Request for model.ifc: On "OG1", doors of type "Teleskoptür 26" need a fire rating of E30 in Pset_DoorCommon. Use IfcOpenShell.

First a look at what the model holds.

```python
import ifcopenshell
import ifcopenshell.util.element

model = ifcopenshell.open("model.ifc")
print(model.schema)
storey = next(s for s in model.by_type("IfcBuildingStorey") if s.Name == "OG1")
doors = [e for e in ifcopenshell.util.element.get_decomposition(storey) if e.is_a("IfcDoor")]
seen = {}
for e in doors:
    element_type = ifcopenshell.util.element.get_type(e)
    key = (element_type.Name if element_type != e and element_type else None, ifcopenshell.util.element.get_pset(e, "Pset_DoorCommon", "FireRating"))
    seen[key] = seen.get(key, 0) + 1
for (name, value), count in sorted(seen.items(), key=str):
    print(count, "x", name, "|", value)
```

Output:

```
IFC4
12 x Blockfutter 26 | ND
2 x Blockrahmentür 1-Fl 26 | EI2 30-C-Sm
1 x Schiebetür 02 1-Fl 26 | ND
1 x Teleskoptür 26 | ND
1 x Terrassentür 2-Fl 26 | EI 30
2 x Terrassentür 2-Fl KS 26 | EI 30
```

```python
import ifcopenshell
import ifcopenshell.api.pset
import ifcopenshell.util.element

model = ifcopenshell.open("model.ifc")

storey = next(s for s in model.by_type("IfcBuildingStorey") if s.Name == "OG1")
doors = [e for e in ifcopenshell.util.element.get_decomposition(storey) if e.is_a("IfcDoor")]

count = 0
for e in doors:
    element_type = ifcopenshell.util.element.get_type(e)
    if element_type in (None, e) or element_type.Name != "Teleskoptür 26":
        continue
    # add_pset returns the element's existing set when there is one.
    pset = ifcopenshell.api.pset.add_pset(model, product=e, name="Pset_DoorCommon")
    ifcopenshell.api.pset.edit_pset(model, pset=pset, properties={"FireRating": "E30"})
    count += 1

print(count, "doors updated")

model.write("model-out.ifc")
```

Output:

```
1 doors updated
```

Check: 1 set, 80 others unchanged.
